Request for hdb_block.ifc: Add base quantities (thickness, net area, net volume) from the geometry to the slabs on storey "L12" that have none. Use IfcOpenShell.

First a look at what the model holds.

```python
import ifcopenshell
import ifcopenshell.util.element
import ifcopenshell.util.unit

model = ifcopenshell.open("hdb_block.ifc")
print(model.schema)
for unit_type in ("LENGTHUNIT", "AREAUNIT", "VOLUMEUNIT"):
    print(unit_type, ifcopenshell.util.unit.calculate_unit_scale(model, unit_type))
storey = next(s for s in model.by_type("IfcBuildingStorey") if s.Name == "L12")
slabs = [e for e in ifcopenshell.util.element.get_decomposition(storey) if e.is_a("IfcSlab")]
for e in sorted(slabs, key=lambda e: e.id()):
    print(e.id(), e.is_a(), e.Name, list(ifcopenshell.util.element.get_psets(e, qtos_only=True)), sep=" | ")
```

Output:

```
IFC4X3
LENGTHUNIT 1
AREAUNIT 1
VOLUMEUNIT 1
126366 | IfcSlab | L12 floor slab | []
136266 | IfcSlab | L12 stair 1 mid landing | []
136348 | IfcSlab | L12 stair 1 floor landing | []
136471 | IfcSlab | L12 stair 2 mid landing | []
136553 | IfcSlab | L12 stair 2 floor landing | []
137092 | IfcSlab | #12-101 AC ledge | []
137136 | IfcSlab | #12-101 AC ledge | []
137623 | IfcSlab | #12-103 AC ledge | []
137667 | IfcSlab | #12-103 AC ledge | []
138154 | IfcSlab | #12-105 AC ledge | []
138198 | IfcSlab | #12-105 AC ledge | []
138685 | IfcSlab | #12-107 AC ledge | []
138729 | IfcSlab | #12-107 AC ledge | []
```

```python
import ifcopenshell
import ifcopenshell.api.pset
import ifcopenshell.geom
import ifcopenshell.util.element
import ifcopenshell.util.shape
import ifcopenshell.util.unit

model = ifcopenshell.open("hdb_block.ifc")
unit_scale = ifcopenshell.util.unit.calculate_unit_scale(model)
area_scale = ifcopenshell.util.unit.calculate_unit_scale(model, "AREAUNIT")
volume_scale = ifcopenshell.util.unit.calculate_unit_scale(model, "VOLUMEUNIT")
settings = ifcopenshell.geom.settings()

storey = next(s for s in model.by_type("IfcBuildingStorey") if s.Name == "L12")
slabs = [e for e in ifcopenshell.util.element.get_decomposition(storey) if e.is_a("IfcSlab")]

for e in sorted(slabs, key=lambda e: e.id()):
    if ifcopenshell.util.element.get_psets(e, qtos_only=True, should_inherit=False):
        continue
    # Geometry comes back in metres, in the element's own axes.
    shape = ifcopenshell.geom.create_shape(settings, e)
    values = {
        "Width": ifcopenshell.util.shape.get_z(shape.geometry) / unit_scale,
        "NetArea": ifcopenshell.util.shape.get_footprint_area(shape.geometry) / area_scale,
        "NetVolume": ifcopenshell.util.shape.get_volume(shape.geometry) / volume_scale,
    }
    qto = ifcopenshell.api.pset.add_qto(model, product=e, name="Qto_SlabBaseQuantities")
    ifcopenshell.api.pset.edit_qto(model, qto=qto, properties=values)
    print(e.id(), {k: round(v, 3) for k, v in values.items()})

model.write("hdb_block_edited.ifc")
```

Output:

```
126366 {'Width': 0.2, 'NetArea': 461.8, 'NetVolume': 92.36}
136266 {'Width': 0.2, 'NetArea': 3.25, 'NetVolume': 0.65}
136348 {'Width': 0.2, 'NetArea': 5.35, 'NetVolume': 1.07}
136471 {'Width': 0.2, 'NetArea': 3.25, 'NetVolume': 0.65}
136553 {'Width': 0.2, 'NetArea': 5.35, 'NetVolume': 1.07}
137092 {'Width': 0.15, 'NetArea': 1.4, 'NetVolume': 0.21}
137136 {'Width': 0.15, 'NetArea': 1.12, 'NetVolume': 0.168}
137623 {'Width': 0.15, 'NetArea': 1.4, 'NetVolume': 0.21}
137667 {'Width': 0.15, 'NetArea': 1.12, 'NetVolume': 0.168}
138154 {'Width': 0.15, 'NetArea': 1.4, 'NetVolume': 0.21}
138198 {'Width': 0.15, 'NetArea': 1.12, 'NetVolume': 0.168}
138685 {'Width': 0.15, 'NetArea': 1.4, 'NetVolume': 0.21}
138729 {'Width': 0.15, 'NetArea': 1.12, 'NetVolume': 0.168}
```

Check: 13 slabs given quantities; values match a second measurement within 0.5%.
